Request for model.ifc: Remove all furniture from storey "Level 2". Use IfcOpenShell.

First a look at what the model holds.

```python
import ifcopenshell
import ifcopenshell.util.element

model = ifcopenshell.open("model.ifc")
print(model.schema)
storey = next(s for s in model.by_type("IfcBuildingStorey") if s.Name == "Level 2")
furniture = [e for e in ifcopenshell.util.element.get_decomposition(storey) if e.is_a("IfcFurnishingElement")]
seen = {}
for e in furniture:
    element_type = ifcopenshell.util.element.get_type(e)
    name = element_type.Name if element_type not in (None, e) else None
    seen[name] = seen.get(name, 0) + 1
for name, count in sorted(seen.items(), key=str):
    print(count, "x", name)
```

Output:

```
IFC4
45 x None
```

```python
import ifcopenshell
import ifcopenshell.api.root
import ifcopenshell.util.element

model = ifcopenshell.open("model.ifc")

storey = next(s for s in model.by_type("IfcBuildingStorey") if s.Name == "Level 2")
furniture = [e for e in ifcopenshell.util.element.get_decomposition(storey) if e.is_a("IfcFurnishingElement")]

for e in furniture:
    ifcopenshell.api.root.remove_product(model, product=e)
print(len(furniture), "removed")

model.write("model_updated.ifc")
```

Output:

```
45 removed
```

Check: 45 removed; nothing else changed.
